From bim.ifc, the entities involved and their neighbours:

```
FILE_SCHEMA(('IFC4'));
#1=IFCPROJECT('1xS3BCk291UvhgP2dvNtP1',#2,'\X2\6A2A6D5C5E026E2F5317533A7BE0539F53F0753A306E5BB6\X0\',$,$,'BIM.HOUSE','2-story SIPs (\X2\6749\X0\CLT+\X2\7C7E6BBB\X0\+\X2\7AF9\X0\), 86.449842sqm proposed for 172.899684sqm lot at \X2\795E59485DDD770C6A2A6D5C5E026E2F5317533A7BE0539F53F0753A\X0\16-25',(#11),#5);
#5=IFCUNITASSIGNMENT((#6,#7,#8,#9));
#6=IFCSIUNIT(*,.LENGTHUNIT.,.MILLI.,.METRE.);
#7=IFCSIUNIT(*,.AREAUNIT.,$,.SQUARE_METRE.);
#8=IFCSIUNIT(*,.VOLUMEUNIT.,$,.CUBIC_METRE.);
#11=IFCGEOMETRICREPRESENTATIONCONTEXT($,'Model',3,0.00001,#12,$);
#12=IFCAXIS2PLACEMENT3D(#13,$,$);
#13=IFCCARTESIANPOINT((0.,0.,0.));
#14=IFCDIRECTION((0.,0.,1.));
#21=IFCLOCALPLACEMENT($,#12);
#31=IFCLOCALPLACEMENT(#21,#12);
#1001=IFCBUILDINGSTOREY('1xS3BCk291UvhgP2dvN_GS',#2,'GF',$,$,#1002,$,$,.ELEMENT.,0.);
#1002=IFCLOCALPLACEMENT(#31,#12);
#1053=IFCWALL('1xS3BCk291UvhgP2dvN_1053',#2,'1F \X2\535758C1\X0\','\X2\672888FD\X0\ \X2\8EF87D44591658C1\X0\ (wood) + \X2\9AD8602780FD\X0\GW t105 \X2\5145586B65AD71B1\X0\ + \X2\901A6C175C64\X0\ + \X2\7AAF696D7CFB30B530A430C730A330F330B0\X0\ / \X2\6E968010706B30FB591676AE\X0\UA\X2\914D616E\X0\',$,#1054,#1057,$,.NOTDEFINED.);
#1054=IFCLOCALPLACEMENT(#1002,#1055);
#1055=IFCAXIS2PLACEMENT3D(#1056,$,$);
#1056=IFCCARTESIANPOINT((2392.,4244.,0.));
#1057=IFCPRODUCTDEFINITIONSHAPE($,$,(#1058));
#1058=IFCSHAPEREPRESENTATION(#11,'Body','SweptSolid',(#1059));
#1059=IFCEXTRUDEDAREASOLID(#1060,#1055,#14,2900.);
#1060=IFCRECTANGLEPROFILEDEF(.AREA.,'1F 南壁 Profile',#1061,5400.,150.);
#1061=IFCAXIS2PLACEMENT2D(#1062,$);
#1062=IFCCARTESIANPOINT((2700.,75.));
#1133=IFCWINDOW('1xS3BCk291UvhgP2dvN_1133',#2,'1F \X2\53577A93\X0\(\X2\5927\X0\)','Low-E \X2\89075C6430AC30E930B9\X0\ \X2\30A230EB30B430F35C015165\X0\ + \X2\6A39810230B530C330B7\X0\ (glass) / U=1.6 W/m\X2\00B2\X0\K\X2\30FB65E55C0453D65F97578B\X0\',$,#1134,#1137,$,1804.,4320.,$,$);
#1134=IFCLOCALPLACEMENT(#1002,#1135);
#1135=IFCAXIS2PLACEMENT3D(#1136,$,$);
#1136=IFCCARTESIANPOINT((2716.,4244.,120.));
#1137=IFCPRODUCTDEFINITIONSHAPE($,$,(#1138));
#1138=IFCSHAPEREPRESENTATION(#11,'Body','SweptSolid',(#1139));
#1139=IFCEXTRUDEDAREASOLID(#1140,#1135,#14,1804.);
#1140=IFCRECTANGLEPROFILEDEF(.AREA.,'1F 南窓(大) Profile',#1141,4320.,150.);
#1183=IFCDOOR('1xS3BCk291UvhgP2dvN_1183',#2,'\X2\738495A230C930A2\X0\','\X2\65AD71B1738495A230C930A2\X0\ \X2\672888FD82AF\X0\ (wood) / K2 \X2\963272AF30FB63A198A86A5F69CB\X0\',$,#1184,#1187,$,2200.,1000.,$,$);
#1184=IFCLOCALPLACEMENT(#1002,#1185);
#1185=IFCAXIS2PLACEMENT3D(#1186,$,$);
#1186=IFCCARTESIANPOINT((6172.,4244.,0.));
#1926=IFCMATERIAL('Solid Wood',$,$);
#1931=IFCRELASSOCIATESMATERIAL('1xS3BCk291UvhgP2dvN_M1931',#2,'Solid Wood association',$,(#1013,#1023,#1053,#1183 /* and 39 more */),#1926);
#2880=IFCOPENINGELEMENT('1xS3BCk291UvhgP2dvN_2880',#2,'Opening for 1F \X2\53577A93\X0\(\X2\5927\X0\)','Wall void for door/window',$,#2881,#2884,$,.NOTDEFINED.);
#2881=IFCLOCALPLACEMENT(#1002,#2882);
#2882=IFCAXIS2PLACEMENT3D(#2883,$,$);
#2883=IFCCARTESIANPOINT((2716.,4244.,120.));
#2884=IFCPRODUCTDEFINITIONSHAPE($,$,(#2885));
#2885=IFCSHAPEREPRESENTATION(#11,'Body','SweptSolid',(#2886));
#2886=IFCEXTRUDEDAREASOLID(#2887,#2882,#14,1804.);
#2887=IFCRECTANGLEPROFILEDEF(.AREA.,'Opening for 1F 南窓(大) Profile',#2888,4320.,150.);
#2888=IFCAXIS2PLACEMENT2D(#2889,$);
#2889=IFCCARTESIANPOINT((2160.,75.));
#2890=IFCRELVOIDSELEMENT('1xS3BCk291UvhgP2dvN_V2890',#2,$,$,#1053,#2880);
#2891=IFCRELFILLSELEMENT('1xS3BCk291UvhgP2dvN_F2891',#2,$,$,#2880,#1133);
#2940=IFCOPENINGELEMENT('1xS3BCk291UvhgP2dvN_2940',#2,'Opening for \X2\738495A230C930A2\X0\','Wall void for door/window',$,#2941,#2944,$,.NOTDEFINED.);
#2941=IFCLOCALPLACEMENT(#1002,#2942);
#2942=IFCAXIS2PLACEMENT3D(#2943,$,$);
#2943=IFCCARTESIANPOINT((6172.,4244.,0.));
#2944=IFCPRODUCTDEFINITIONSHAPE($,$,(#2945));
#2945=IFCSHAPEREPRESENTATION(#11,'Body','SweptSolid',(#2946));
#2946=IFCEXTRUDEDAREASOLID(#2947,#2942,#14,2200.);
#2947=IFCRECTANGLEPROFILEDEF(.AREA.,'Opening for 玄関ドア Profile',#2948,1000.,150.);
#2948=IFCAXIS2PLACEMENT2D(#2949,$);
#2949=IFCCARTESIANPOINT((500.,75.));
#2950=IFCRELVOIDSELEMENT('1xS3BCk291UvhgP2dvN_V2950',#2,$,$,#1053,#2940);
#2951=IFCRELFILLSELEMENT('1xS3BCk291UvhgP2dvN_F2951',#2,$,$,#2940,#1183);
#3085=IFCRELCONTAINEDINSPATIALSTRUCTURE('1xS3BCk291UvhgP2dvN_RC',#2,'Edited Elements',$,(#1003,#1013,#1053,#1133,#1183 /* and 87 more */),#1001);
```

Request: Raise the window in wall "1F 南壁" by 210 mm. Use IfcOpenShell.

```python
import numpy as np
import ifcopenshell
import ifcopenshell.api.geometry
import ifcopenshell.util.placement
import ifcopenshell.util.unit

model = ifcopenshell.open("bim.ifc")
unit_scale = ifcopenshell.util.unit.calculate_unit_scale(model)

window = model.by_guid("1xS3BCk291UvhgP2dvN_1133")
opening = window.FillsVoids[0].RelatingOpeningElement
dz = 0.21 / unit_scale

shift = np.array([0.0, 0.0, dz])
# The window is not placed relative to its opening, so move both.
for product in (opening, window):
    matrix = ifcopenshell.util.placement.get_local_placement(product.ObjectPlacement)
    matrix[:3, 3] += shift
    ifcopenshell.api.geometry.edit_object_placement(model, product=product, matrix=matrix, is_si=False)

print(f"moved by {dz * unit_scale:+.3f} m")

model.write("bim_updated.ifc")
```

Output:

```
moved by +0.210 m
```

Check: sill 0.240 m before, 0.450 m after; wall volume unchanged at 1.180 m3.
